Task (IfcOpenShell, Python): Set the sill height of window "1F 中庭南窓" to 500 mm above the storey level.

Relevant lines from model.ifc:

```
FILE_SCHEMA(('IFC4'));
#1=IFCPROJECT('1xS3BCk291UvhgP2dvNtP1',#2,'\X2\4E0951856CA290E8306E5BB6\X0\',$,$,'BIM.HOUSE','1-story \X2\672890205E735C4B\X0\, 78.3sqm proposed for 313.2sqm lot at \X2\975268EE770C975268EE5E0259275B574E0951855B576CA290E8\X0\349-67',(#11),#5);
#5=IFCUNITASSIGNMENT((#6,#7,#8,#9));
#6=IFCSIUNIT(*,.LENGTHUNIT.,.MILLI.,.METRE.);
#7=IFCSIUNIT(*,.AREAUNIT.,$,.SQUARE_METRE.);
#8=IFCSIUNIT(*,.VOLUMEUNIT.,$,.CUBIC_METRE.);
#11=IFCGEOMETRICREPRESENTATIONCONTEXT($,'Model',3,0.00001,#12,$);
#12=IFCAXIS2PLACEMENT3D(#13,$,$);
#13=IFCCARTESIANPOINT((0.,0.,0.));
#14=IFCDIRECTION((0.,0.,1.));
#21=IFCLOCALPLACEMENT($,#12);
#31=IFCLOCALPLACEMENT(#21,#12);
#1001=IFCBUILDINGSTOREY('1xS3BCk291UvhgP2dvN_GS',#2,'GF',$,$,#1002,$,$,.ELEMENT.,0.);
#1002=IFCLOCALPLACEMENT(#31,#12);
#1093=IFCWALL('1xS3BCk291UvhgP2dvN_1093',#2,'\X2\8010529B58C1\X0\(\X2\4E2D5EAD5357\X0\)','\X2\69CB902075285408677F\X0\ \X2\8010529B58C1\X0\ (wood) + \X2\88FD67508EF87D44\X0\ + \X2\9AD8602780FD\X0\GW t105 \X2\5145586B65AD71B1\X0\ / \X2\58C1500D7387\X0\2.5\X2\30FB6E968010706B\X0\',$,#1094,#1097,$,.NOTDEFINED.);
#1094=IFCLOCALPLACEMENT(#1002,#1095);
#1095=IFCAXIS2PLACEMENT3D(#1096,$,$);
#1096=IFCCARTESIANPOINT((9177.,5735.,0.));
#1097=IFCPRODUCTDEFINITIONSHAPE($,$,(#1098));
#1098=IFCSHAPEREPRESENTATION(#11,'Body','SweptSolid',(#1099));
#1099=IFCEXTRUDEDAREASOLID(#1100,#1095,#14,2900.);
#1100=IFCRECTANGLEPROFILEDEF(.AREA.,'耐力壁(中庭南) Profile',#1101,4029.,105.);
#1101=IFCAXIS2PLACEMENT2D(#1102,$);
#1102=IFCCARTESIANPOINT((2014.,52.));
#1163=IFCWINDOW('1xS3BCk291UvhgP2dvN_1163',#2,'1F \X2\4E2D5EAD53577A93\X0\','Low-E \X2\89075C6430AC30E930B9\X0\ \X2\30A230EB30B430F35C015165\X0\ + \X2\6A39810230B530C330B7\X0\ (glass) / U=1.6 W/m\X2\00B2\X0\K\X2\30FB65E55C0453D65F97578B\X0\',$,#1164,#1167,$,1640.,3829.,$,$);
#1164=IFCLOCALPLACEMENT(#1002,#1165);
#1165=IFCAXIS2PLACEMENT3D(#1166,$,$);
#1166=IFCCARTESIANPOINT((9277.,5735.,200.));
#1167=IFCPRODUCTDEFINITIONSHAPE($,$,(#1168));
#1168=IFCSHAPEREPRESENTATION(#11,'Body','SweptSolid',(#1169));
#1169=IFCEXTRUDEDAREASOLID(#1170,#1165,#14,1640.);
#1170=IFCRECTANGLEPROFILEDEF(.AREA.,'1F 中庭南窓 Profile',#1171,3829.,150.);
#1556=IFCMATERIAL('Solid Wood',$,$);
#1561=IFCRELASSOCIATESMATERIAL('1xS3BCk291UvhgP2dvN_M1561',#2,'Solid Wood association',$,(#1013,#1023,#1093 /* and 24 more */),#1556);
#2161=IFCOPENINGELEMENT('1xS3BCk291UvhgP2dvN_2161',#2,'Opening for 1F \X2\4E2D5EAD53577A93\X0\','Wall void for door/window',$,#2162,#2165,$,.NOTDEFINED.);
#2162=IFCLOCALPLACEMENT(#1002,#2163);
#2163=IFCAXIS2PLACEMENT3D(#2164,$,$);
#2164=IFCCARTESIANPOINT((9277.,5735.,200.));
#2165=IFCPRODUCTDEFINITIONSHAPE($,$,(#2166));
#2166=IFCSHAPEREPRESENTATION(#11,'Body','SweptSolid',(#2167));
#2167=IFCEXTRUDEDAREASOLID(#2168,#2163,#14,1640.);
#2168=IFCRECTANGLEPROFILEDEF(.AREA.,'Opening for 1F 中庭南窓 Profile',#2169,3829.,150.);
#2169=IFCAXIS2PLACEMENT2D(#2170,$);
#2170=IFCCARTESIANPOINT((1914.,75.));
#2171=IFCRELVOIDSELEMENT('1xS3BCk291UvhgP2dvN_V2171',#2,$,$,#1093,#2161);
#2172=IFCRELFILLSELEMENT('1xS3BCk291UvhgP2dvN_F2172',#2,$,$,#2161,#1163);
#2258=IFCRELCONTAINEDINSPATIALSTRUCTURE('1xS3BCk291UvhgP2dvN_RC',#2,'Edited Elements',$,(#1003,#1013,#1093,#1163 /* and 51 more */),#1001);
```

```python
import numpy as np
import ifcopenshell
import ifcopenshell.api.geometry
import ifcopenshell.geom
import ifcopenshell.util.element
import ifcopenshell.util.placement
import ifcopenshell.util.shape
import ifcopenshell.util.unit

model = ifcopenshell.open("model.ifc")
unit_scale = ifcopenshell.util.unit.calculate_unit_scale(model)

window = model.by_id(1163)
opening = window.FillsVoids[0].RelatingOpeningElement
storey = ifcopenshell.util.element.get_container(window, ifc_class="IfcBuildingStorey")
level = ifcopenshell.util.placement.get_local_placement(storey.ObjectPlacement)[2, 3]

# The opening's origin need not be at the sill, so measure its lowest point.
shape = ifcopenshell.geom.create_shape(ifcopenshell.geom.settings(), opening)
bottom = ifcopenshell.util.shape.get_shape_bottom_elevation(shape, shape.geometry) / unit_scale
dz = level + 0.5 / unit_scale - bottom

shift = np.array([0.0, 0.0, dz])
# The window is not placed relative to its opening, so move both.
for product in (opening, window):
    matrix = ifcopenshell.util.placement.get_local_placement(product.ObjectPlacement)
    matrix[:3, 3] += shift
    ifcopenshell.api.geometry.edit_object_placement(model, product=product, matrix=matrix, is_si=False)

print(f"moved by {dz * unit_scale:+.3f} m")

model.write("model_edited.ifc")
```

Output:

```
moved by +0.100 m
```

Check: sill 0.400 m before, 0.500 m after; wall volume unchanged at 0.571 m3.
